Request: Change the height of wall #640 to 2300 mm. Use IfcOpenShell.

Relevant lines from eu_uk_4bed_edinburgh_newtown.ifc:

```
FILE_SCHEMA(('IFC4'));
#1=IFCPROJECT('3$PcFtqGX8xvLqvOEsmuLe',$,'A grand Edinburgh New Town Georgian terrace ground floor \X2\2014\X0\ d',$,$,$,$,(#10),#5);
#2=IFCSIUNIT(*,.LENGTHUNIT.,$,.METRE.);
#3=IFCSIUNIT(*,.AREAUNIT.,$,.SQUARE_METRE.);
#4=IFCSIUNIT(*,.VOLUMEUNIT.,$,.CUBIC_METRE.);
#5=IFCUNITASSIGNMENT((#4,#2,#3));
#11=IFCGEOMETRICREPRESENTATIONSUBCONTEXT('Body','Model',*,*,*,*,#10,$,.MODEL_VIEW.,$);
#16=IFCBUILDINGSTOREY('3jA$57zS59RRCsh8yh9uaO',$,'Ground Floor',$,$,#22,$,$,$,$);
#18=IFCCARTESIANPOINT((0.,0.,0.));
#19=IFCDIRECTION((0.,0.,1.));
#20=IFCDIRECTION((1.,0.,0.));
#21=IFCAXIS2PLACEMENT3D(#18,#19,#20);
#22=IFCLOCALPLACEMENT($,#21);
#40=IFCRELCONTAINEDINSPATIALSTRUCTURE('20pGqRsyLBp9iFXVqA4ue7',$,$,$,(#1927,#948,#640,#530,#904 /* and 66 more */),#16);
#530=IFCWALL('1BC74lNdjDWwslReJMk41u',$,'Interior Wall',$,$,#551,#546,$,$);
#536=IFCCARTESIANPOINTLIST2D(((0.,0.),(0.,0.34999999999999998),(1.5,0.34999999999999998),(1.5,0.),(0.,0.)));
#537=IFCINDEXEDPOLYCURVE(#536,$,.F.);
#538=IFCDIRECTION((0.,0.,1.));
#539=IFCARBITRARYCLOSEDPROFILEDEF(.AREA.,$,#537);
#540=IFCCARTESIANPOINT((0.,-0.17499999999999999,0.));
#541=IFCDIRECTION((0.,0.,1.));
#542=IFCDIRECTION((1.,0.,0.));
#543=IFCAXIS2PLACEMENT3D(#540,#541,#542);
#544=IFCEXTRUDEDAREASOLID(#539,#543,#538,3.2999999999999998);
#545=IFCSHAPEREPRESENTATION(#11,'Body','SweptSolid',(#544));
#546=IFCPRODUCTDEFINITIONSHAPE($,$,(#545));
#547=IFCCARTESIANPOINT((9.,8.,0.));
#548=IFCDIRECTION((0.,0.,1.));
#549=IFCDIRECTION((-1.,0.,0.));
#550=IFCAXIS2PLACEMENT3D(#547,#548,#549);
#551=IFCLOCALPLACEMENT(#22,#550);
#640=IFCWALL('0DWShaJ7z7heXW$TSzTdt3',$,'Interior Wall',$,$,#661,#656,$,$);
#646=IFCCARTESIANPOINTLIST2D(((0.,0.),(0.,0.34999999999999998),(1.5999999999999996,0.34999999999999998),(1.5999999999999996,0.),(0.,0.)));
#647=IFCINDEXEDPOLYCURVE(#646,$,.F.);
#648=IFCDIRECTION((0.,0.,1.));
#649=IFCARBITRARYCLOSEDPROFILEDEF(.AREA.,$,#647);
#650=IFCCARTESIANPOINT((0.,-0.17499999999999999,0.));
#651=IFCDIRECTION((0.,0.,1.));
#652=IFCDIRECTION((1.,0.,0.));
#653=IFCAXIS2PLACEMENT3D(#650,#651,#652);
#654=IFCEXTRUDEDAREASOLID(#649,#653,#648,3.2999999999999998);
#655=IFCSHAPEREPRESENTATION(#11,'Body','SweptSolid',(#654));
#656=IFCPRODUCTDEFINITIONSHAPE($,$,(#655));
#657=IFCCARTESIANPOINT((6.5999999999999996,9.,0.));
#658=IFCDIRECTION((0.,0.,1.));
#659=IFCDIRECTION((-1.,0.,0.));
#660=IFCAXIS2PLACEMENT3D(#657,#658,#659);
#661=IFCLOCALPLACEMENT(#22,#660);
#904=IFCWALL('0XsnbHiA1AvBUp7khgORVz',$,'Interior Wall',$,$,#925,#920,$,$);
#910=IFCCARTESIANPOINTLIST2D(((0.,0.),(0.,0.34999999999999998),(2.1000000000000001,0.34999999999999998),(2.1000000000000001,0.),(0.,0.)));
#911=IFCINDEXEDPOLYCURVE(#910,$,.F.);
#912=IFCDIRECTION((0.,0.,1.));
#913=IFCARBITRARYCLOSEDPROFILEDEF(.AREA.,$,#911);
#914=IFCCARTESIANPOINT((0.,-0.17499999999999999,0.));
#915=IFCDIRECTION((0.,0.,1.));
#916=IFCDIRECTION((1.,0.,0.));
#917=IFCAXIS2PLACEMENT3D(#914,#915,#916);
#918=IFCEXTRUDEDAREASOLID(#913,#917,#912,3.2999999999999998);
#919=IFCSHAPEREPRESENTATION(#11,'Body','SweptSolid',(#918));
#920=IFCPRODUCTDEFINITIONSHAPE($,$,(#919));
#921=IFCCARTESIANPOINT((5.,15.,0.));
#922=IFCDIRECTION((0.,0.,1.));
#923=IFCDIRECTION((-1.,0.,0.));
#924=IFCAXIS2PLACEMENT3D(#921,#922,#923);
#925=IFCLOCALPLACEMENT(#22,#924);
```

```python
import ifcopenshell
import ifcopenshell.geom
import ifcopenshell.util.representation
import ifcopenshell.util.shape
import ifcopenshell.util.unit

model = ifcopenshell.open("eu_uk_4bed_edinburgh_newtown.ifc")
unit_scale = ifcopenshell.util.unit.calculate_unit_scale(model)
settings = ifcopenshell.geom.settings()


def volume(element):
    """Net volume in cubic metres, openings subtracted."""
    shape = ifcopenshell.geom.create_shape(settings, element)
    return ifcopenshell.util.shape.get_volume(shape.geometry)


wall = model.by_guid("0DWShaJ7z7heXW$TSzTdt3")
before = volume(wall)

body = ifcopenshell.util.representation.get_representation(wall, "Model", "Body")
solid = body.Items[0]
old_height = solid.Depth
solid.Depth = 2.3 / unit_scale
after = volume(wall)

print(f"height {old_height:g} -> {solid.Depth:g}, volume {before:.3f} -> {after:.3f} m3")

model.write("eu_uk_4bed_edinburgh_newtown_edited.ifc")
```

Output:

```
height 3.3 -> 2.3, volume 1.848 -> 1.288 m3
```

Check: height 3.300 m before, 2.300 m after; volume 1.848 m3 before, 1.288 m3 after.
